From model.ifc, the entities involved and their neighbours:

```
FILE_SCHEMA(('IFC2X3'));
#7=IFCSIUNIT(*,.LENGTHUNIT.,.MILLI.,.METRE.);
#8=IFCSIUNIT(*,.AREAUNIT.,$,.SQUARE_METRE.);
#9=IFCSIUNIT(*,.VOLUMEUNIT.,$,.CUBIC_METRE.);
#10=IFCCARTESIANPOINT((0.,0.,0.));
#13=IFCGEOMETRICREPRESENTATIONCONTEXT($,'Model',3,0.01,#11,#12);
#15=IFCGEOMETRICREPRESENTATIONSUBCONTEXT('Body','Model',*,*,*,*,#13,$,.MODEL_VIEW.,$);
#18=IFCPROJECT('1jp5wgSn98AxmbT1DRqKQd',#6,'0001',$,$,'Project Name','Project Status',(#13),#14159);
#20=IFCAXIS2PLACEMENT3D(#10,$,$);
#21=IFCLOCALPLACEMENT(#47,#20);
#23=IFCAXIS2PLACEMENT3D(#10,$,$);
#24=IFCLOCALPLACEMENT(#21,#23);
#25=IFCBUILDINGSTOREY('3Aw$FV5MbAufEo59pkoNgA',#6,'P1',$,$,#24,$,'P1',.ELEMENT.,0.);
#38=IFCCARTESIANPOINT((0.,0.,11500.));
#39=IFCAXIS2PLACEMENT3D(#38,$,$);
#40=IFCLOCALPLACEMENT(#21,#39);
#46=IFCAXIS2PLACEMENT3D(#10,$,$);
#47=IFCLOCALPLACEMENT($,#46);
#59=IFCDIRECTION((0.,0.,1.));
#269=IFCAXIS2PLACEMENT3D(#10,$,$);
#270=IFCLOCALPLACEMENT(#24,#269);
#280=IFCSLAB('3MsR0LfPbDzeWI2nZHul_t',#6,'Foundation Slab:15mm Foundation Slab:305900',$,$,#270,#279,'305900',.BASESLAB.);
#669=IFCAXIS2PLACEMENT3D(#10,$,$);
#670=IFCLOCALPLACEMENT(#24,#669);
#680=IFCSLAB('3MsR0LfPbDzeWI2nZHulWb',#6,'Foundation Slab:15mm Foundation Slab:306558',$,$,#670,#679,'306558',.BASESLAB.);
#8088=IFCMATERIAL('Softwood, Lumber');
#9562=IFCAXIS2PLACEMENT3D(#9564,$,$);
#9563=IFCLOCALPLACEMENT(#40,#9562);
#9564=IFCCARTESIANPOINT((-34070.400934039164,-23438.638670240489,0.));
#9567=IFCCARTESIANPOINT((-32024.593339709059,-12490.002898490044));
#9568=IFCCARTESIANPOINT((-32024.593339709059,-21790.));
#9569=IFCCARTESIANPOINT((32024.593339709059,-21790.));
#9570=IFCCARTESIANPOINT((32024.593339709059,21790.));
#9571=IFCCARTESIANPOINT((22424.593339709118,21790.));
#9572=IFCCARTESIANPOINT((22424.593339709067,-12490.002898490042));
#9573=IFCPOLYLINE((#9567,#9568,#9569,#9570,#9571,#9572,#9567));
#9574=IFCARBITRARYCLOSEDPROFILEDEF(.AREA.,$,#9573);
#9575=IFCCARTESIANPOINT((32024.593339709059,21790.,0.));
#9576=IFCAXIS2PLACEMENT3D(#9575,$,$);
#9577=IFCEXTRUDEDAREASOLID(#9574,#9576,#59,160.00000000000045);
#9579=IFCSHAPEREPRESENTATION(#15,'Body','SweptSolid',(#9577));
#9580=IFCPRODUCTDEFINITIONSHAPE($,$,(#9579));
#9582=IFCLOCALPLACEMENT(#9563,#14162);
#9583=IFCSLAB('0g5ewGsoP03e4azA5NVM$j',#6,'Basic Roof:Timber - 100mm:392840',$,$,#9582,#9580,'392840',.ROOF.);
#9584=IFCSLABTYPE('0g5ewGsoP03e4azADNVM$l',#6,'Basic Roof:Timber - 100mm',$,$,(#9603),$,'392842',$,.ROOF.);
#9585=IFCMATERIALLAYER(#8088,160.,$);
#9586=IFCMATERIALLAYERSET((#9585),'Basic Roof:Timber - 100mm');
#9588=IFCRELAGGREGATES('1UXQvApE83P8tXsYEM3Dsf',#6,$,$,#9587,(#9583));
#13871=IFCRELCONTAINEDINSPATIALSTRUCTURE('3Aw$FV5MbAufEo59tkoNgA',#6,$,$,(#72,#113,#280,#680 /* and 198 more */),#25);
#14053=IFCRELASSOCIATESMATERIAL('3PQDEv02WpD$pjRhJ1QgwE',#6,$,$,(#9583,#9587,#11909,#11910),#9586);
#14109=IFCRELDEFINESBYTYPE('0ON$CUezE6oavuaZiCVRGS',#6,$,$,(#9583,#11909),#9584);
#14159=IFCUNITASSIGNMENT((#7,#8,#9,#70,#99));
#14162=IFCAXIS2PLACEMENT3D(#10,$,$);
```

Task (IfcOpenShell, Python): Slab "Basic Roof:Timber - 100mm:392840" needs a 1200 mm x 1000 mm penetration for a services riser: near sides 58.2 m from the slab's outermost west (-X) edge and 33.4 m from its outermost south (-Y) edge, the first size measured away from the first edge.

```python
import numpy as np
import ifcopenshell
import ifcopenshell.api.feature
import ifcopenshell.api.geometry
import ifcopenshell.api.root
import ifcopenshell.geom
import ifcopenshell.util.placement
import ifcopenshell.util.representation
import ifcopenshell.util.shape
import ifcopenshell.util.unit

model = ifcopenshell.open("model.ifc")
unit_scale = ifcopenshell.util.unit.calculate_unit_scale(model)
settings = ifcopenshell.geom.settings()


def volume(element):
    """Net volume in cubic metres, openings subtracted."""
    shape = ifcopenshell.geom.create_shape(settings, element)
    return ifcopenshell.util.shape.get_volume(shape.geometry)


slab = model.by_guid("0g5ewGsoP03e4azA5NVM$j")
before = volume(slab)

# Extent in the slab's own axes, in metres. The edges named are its -X and -Y sides.
slab_shape = ifcopenshell.geom.create_shape(settings, slab)
vertices = ifcopenshell.util.shape.get_vertices(slab_shape.geometry)
x_min, y_min, bottom = vertices.min(axis=0)
top = vertices[:, 2].max()

opening = ifcopenshell.api.root.create_entity(model, ifc_class="IfcOpeningElement", name="Services riser opening")
context = ifcopenshell.util.representation.get_context(model, "Model", "Body", "MODEL_VIEW")
width, depth = 1.2, 1
outline = [(0.0, 0.0), (width, 0.0), (width, depth), (0.0, depth), (0.0, 0.0)]
# Overshoot both faces by 50 mm so the cut is clean.
shape = ifcopenshell.api.geometry.add_slab_representation(
    model, context=context, depth=top - bottom + 0.1, polyline=outline
)
ifcopenshell.api.geometry.assign_representation(model, product=opening, representation=shape)

matrix = ifcopenshell.util.placement.get_local_placement(slab.ObjectPlacement)
matrix[:, 3] = matrix @ np.append(np.array([x_min + 58.2, y_min + 33.4, bottom - 0.05]) / unit_scale, 1.0)
ifcopenshell.api.geometry.edit_object_placement(model, product=opening, matrix=matrix, is_si=False)
ifcopenshell.api.feature.add_feature(model, feature=opening, element=slab)

after = volume(slab)

print(f"slab volume {before:.3f} -> {after:.3f} m3")

model.write("model-out.ifc")
```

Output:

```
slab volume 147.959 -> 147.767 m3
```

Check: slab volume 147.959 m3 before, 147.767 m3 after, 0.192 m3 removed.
